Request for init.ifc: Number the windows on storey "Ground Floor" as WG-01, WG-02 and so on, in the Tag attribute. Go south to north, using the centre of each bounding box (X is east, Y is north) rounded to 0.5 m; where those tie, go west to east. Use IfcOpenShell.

First a look at what the model holds.

```python
import ifcopenshell
import ifcopenshell.util.element
import ifcopenshell.util.placement

model = ifcopenshell.open("init.ifc")
print(model.schema)
storey = next(s for s in model.by_type("IfcBuildingStorey") if s.Name == "Ground Floor")
windows = [e for e in ifcopenshell.util.element.get_decomposition(storey) if e.is_a("IfcWindow")]
for e in sorted(windows, key=lambda e: e.id()):
    origin = ifcopenshell.util.placement.get_local_placement(e.ObjectPlacement)[:3, 3]
    print(e.id(), e.Tag, e.Name, origin.round(2) + 0.0, sep=" | ")
```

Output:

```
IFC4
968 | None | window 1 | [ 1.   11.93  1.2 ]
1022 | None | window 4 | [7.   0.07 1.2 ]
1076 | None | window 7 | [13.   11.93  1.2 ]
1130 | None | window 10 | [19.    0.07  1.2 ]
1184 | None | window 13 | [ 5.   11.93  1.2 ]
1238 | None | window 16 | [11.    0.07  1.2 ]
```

```python
import ifcopenshell
import ifcopenshell.geom
import ifcopenshell.util.element
import ifcopenshell.util.shape

model = ifcopenshell.open("init.ifc")
settings = ifcopenshell.geom.settings()
settings.set("use-world-coords", True)


def centre(element):
    shape = ifcopenshell.geom.create_shape(settings, element)
    return ifcopenshell.util.shape.get_bbox_centroid(shape.geometry)


storey = next(s for s in model.by_type("IfcBuildingStorey") if s.Name == "Ground Floor")
windows = [e for e in ifcopenshell.util.element.get_decomposition(storey) if e.is_a("IfcWindow")]

# Insertion points can sit at a corner or the storey origin, so sort by the geometry (in metres).
centres = {e: centre(e) for e in windows}
windows.sort(key=lambda e: (round(centres[e][1] / 0.5), centres[e][0]))

for i, e in enumerate(windows, start=1):
    number = f"WG-{i:02d}"
    e.Tag = number
    print(e.id(), number)

model.write("init-out.ifc")
```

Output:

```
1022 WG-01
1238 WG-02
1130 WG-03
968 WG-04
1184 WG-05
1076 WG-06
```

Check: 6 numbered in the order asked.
